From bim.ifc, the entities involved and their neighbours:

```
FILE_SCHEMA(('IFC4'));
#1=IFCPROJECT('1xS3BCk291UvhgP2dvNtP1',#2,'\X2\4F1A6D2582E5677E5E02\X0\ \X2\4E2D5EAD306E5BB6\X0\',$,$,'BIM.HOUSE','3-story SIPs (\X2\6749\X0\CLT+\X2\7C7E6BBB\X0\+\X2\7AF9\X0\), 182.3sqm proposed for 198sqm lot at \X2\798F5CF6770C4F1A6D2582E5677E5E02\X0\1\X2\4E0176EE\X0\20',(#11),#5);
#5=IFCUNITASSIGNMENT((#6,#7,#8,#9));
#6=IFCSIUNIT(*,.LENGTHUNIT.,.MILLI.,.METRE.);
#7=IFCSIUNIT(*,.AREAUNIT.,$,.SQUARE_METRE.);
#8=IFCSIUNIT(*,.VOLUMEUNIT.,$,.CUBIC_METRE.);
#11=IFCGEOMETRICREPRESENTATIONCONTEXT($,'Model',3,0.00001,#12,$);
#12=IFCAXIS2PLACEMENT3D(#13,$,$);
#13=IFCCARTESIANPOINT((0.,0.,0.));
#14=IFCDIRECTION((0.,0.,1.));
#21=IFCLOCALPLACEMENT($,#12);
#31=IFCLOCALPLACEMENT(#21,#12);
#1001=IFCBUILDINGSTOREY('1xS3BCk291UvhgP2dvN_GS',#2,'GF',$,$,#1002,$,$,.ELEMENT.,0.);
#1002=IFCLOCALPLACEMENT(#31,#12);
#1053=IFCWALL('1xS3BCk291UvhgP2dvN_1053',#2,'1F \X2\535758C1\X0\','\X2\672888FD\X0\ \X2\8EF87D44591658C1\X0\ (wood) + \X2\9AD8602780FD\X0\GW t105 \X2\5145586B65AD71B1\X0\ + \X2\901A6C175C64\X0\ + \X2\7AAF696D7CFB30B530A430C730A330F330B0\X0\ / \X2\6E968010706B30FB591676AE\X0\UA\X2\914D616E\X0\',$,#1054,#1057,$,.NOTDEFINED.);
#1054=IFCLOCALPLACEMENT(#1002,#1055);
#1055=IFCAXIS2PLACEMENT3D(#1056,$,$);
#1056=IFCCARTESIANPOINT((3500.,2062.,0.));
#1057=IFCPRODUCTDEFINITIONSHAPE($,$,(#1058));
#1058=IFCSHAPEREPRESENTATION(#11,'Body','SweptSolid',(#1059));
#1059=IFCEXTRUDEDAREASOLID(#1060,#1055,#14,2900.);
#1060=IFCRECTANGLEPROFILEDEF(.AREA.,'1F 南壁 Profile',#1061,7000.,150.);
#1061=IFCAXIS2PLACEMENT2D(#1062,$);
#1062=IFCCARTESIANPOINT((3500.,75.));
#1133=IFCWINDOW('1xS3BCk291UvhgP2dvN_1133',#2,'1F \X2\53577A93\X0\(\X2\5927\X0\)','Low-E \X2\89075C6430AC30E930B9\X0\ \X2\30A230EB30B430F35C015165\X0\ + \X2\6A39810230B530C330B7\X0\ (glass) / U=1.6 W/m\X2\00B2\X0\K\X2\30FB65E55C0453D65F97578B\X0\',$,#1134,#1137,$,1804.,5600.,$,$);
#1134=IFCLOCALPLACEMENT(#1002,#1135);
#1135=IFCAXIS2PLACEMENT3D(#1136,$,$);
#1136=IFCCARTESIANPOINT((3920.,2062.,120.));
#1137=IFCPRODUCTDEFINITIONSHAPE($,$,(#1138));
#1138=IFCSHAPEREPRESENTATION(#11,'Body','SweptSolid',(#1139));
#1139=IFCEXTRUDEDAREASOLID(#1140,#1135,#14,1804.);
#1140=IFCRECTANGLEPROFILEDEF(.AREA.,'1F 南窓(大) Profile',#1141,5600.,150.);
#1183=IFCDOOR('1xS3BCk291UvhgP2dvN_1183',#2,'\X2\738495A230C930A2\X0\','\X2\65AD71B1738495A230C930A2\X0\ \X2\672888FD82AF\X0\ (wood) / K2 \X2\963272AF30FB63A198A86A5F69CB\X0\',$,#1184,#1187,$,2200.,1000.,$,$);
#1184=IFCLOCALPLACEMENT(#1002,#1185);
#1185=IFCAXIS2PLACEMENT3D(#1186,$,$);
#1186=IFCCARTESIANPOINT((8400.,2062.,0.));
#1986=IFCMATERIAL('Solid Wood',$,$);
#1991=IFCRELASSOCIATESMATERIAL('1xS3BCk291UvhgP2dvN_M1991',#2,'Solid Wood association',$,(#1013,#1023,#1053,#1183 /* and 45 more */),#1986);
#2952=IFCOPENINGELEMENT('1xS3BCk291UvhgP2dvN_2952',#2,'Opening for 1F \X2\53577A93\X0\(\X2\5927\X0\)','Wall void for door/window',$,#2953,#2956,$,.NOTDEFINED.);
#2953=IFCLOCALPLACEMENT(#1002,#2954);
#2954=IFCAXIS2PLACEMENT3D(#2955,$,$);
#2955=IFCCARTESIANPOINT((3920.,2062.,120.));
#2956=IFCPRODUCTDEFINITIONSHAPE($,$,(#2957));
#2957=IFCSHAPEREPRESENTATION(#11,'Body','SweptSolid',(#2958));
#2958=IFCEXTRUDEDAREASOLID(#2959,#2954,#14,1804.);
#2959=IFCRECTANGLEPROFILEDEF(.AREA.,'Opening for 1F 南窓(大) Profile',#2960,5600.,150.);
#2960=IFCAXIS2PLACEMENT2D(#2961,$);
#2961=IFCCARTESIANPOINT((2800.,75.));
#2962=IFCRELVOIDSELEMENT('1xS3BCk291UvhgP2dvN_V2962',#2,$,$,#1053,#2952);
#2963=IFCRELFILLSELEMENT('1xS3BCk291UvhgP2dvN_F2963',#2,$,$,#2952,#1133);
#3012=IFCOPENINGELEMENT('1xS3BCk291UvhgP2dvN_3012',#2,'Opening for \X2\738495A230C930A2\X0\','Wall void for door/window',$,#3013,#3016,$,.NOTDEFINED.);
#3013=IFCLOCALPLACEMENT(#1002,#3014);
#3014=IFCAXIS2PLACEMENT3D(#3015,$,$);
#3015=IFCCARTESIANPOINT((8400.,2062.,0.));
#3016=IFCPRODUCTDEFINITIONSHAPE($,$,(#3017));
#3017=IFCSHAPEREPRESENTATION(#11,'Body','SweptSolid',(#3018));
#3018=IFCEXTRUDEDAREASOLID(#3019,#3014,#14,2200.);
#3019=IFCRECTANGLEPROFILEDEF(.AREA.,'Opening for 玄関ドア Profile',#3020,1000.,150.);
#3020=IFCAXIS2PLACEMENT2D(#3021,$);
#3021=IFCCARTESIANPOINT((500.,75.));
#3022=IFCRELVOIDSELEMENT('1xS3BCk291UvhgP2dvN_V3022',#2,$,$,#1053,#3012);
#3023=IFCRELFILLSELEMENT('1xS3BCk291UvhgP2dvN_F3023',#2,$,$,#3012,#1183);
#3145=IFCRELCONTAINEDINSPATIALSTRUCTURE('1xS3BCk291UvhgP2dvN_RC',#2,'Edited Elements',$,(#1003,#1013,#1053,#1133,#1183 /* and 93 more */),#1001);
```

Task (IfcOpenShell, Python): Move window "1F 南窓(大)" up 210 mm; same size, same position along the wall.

```python
import numpy as np
import ifcopenshell
import ifcopenshell.api.geometry
import ifcopenshell.util.placement
import ifcopenshell.util.unit

model = ifcopenshell.open("bim.ifc")
unit_scale = ifcopenshell.util.unit.calculate_unit_scale(model)

window = model.by_id(1133)
opening = window.FillsVoids[0].RelatingOpeningElement
dz = 210.0

shift = np.array([0.0, 0.0, dz])
# The window is not placed relative to its opening, so move both.
for product in (opening, window):
    matrix = ifcopenshell.util.placement.get_local_placement(product.ObjectPlacement)
    matrix[:3, 3] += shift
    ifcopenshell.api.geometry.edit_object_placement(model, product=product, matrix=matrix, is_si=False)

print(f"moved by {dz * unit_scale:+.3f} m")

model.write("bim_rev.ifc")
```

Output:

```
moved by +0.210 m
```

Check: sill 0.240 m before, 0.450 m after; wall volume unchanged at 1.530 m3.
